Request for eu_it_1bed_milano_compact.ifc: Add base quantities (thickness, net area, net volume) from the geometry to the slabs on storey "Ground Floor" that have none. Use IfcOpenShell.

First a look at what the model holds.

```python
import ifcopenshell
import ifcopenshell.util.element
import ifcopenshell.util.unit

model = ifcopenshell.open("eu_it_1bed_milano_compact.ifc")
print(model.schema)
for unit_type in ("LENGTHUNIT", "AREAUNIT", "VOLUMEUNIT"):
    print(unit_type, ifcopenshell.util.unit.calculate_unit_scale(model, unit_type))
storey = next(s for s in model.by_type("IfcBuildingStorey") if s.Name == "Ground Floor")
slabs = [e for e in ifcopenshell.util.element.get_decomposition(storey) if e.is_a("IfcSlab")]
for e in sorted(slabs, key=lambda e: e.id()):
    print(e.id(), e.is_a(), e.Name, list(ifcopenshell.util.element.get_psets(e, qtos_only=True)), sep=" | ")
```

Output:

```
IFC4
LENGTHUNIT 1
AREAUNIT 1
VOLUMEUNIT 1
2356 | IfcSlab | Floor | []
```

```python
import ifcopenshell
import ifcopenshell.api.pset
import ifcopenshell.geom
import ifcopenshell.util.element
import ifcopenshell.util.shape
import ifcopenshell.util.unit

model = ifcopenshell.open("eu_it_1bed_milano_compact.ifc")
unit_scale = ifcopenshell.util.unit.calculate_unit_scale(model)
area_scale = ifcopenshell.util.unit.calculate_unit_scale(model, "AREAUNIT")
volume_scale = ifcopenshell.util.unit.calculate_unit_scale(model, "VOLUMEUNIT")
settings = ifcopenshell.geom.settings()

storey = next(s for s in model.by_type("IfcBuildingStorey") if s.Name == "Ground Floor")
slabs = [e for e in ifcopenshell.util.element.get_decomposition(storey) if e.is_a("IfcSlab")]

for e in sorted(slabs, key=lambda e: e.id()):
    if ifcopenshell.util.element.get_psets(e, qtos_only=True, should_inherit=False):
        continue
    # Geometry comes back in metres, in the element's own axes.
    shape = ifcopenshell.geom.create_shape(settings, e)
    values = {
        "Width": ifcopenshell.util.shape.get_z(shape.geometry) / unit_scale,
        "NetArea": ifcopenshell.util.shape.get_footprint_area(shape.geometry) / area_scale,
        "NetVolume": ifcopenshell.util.shape.get_volume(shape.geometry) / volume_scale,
    }
    qto = ifcopenshell.api.pset.add_qto(model, product=e, name="Qto_SlabBaseQuantities")
    ifcopenshell.api.pset.edit_qto(model, qto=qto, properties=values)
    print(e.id(), {k: round(v, 3) for k, v in values.items()})

model.write("eu_it_1bed_milano_compact_rev.ifc")
```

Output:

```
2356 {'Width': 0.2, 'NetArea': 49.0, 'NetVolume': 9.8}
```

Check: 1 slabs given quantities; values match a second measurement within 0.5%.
